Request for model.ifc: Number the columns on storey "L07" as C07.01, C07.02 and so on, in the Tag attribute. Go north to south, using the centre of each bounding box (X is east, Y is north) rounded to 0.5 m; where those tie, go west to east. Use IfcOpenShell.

First a look at what the model holds.

```python
import ifcopenshell
import ifcopenshell.util.element
import ifcopenshell.util.placement

model = ifcopenshell.open("model.ifc")
print(model.schema)
storey = next(s for s in model.by_type("IfcBuildingStorey") if s.Name == "L07")
columns = [e for e in ifcopenshell.util.element.get_decomposition(storey) if e.is_a("IfcColumn")]
for e in sorted(columns, key=lambda e: e.id()):
    origin = ifcopenshell.util.placement.get_local_placement(e.ObjectPlacement)[:3, 3]
    print(e.id(), e.Tag, e.Name, origin.round(2) + 0.0, sep=" | ")
```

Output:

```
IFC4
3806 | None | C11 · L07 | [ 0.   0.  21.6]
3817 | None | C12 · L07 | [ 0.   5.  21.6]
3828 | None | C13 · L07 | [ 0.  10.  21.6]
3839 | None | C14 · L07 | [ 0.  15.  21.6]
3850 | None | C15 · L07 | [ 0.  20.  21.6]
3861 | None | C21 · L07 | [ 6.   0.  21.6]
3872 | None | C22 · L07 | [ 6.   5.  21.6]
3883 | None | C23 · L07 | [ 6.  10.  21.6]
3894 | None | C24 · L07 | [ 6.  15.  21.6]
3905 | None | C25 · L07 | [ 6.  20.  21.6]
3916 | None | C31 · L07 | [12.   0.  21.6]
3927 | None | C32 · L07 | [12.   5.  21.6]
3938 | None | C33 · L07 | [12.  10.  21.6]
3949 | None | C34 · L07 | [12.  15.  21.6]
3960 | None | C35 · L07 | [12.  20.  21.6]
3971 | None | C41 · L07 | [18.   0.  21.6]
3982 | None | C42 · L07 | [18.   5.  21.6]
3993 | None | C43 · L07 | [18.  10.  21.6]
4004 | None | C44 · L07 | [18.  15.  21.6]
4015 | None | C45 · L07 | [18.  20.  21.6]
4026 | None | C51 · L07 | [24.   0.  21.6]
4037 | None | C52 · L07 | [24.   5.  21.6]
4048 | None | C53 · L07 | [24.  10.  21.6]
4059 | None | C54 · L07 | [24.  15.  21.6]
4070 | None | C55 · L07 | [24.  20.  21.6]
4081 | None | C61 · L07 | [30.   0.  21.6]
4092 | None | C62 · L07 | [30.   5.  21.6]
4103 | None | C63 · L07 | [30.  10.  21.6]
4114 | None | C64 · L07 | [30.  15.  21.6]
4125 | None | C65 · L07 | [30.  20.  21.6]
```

```python
import ifcopenshell
import ifcopenshell.geom
import ifcopenshell.util.element
import ifcopenshell.util.shape

model = ifcopenshell.open("model.ifc")
settings = ifcopenshell.geom.settings()
settings.set("use-world-coords", True)


def centre(element):
    shape = ifcopenshell.geom.create_shape(settings, element)
    return ifcopenshell.util.shape.get_bbox_centroid(shape.geometry)


storey = next(s for s in model.by_type("IfcBuildingStorey") if s.Name == "L07")
columns = [e for e in ifcopenshell.util.element.get_decomposition(storey) if e.is_a("IfcColumn")]

# Insertion points can sit at a corner or the storey origin, so sort by the geometry (in metres).
centres = {e: centre(e) for e in columns}
columns.sort(key=lambda e: (-round(centres[e][1] / 0.5), centres[e][0]))

for i, e in enumerate(columns, start=1):
    number = f"C07.{i:02d}"
    e.Tag = number
    print(e.id(), number)

model.write("model-out.ifc")
```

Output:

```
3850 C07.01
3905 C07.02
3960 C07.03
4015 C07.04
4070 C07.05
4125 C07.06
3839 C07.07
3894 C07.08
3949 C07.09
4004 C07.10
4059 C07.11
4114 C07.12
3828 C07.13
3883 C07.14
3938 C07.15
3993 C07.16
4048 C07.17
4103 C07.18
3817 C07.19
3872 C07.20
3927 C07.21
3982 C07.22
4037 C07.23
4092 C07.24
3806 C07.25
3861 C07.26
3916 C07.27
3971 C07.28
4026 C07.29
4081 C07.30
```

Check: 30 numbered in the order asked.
